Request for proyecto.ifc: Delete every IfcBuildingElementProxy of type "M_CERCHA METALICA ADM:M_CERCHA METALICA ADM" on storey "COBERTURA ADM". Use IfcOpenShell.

First a look at what the model holds.

```python
import ifcopenshell
import ifcopenshell.util.element

model = ifcopenshell.open("proyecto.ifc")
print(model.schema)
storey = next(s for s in model.by_type("IfcBuildingStorey") if s.Name == "COBERTURA ADM")
proxies = [e for e in ifcopenshell.util.element.get_decomposition(storey) if e.is_a("IfcBuildingElementProxy")]
seen = {}
for e in proxies:
    element_type = ifcopenshell.util.element.get_type(e)
    name = element_type.Name if element_type not in (None, e) else None
    seen[name] = seen.get(name, 0) + 1
for name, count in sorted(seen.items(), key=str):
    print(count, "x", name)
```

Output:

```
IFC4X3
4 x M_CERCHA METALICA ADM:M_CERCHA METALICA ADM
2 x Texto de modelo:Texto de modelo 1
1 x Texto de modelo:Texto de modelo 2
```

```python
import ifcopenshell
import ifcopenshell.api.root
import ifcopenshell.util.element

model = ifcopenshell.open("proyecto.ifc")

storey = next(s for s in model.by_type("IfcBuildingStorey") if s.Name == "COBERTURA ADM")
proxies = [e for e in ifcopenshell.util.element.get_decomposition(storey) if e.is_a("IfcBuildingElementProxy")]
targets = [e for e in proxies if (t := ifcopenshell.util.element.get_type(e)) not in (None, e) and t.Name == "M_CERCHA METALICA ADM:M_CERCHA METALICA ADM"]

for e in targets:
    ifcopenshell.api.root.remove_product(model, product=e)
print(len(targets), "removed")

model.write("proyecto_rev.ifc")
```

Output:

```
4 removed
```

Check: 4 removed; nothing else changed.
